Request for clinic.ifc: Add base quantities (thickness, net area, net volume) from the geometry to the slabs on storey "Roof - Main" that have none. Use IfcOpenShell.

First a look at what the model holds.

```python
import ifcopenshell
import ifcopenshell.util.element
import ifcopenshell.util.unit

model = ifcopenshell.open("clinic.ifc")
print(model.schema)
for unit_type in ("LENGTHUNIT", "AREAUNIT", "VOLUMEUNIT"):
    print(unit_type, ifcopenshell.util.unit.calculate_unit_scale(model, unit_type))
storey = next(s for s in model.by_type("IfcBuildingStorey") if s.Name == "Roof - Main")
slabs = [e for e in ifcopenshell.util.element.get_decomposition(storey) if e.is_a("IfcSlab")]
for e in sorted(slabs, key=lambda e: e.id()):
    print(e.id(), e.is_a(), e.Name, list(ifcopenshell.util.element.get_psets(e, qtos_only=True)), sep=" | ")
```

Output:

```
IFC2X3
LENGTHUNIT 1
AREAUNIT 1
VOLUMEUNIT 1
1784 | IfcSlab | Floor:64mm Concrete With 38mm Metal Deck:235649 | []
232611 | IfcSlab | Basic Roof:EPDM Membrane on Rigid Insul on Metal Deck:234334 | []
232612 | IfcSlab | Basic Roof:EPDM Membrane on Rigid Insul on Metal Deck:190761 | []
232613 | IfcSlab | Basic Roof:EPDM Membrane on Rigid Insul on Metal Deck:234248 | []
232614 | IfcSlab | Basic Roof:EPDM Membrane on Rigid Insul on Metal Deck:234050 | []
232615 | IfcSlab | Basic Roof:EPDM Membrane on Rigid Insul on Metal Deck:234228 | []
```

```python
import ifcopenshell
import ifcopenshell.api.pset
import ifcopenshell.geom
import ifcopenshell.util.element
import ifcopenshell.util.shape
import ifcopenshell.util.unit

model = ifcopenshell.open("clinic.ifc")
unit_scale = ifcopenshell.util.unit.calculate_unit_scale(model)
area_scale = ifcopenshell.util.unit.calculate_unit_scale(model, "AREAUNIT")
volume_scale = ifcopenshell.util.unit.calculate_unit_scale(model, "VOLUMEUNIT")
settings = ifcopenshell.geom.settings()

storey = next(s for s in model.by_type("IfcBuildingStorey") if s.Name == "Roof - Main")
slabs = [e for e in ifcopenshell.util.element.get_decomposition(storey) if e.is_a("IfcSlab")]

for e in sorted(slabs, key=lambda e: e.id()):
    if ifcopenshell.util.element.get_psets(e, qtos_only=True, should_inherit=False):
        continue
    # Geometry comes back in metres, in the element's own axes.
    shape = ifcopenshell.geom.create_shape(settings, e)
    values = {
        "Width": ifcopenshell.util.shape.get_z(shape.geometry) / unit_scale,
        "NetArea": ifcopenshell.util.shape.get_footprint_area(shape.geometry) / area_scale,
        "NetVolume": ifcopenshell.util.shape.get_volume(shape.geometry) / volume_scale,
    }
    qto = ifcopenshell.api.pset.add_qto(model, product=e, name="BaseQuantities")
    ifcopenshell.api.pset.edit_qto(model, qto=qto, properties=values)
    print(e.id(), {k: round(v, 3) for k, v in values.items()})

model.write("clinic_updated.ifc")
```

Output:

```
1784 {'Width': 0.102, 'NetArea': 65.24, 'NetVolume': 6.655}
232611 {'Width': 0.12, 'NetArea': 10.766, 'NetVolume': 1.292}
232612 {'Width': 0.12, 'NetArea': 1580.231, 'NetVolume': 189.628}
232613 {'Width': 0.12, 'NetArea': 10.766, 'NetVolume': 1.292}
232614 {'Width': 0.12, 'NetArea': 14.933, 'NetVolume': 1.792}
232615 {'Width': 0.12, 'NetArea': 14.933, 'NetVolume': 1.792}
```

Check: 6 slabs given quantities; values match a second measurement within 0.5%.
